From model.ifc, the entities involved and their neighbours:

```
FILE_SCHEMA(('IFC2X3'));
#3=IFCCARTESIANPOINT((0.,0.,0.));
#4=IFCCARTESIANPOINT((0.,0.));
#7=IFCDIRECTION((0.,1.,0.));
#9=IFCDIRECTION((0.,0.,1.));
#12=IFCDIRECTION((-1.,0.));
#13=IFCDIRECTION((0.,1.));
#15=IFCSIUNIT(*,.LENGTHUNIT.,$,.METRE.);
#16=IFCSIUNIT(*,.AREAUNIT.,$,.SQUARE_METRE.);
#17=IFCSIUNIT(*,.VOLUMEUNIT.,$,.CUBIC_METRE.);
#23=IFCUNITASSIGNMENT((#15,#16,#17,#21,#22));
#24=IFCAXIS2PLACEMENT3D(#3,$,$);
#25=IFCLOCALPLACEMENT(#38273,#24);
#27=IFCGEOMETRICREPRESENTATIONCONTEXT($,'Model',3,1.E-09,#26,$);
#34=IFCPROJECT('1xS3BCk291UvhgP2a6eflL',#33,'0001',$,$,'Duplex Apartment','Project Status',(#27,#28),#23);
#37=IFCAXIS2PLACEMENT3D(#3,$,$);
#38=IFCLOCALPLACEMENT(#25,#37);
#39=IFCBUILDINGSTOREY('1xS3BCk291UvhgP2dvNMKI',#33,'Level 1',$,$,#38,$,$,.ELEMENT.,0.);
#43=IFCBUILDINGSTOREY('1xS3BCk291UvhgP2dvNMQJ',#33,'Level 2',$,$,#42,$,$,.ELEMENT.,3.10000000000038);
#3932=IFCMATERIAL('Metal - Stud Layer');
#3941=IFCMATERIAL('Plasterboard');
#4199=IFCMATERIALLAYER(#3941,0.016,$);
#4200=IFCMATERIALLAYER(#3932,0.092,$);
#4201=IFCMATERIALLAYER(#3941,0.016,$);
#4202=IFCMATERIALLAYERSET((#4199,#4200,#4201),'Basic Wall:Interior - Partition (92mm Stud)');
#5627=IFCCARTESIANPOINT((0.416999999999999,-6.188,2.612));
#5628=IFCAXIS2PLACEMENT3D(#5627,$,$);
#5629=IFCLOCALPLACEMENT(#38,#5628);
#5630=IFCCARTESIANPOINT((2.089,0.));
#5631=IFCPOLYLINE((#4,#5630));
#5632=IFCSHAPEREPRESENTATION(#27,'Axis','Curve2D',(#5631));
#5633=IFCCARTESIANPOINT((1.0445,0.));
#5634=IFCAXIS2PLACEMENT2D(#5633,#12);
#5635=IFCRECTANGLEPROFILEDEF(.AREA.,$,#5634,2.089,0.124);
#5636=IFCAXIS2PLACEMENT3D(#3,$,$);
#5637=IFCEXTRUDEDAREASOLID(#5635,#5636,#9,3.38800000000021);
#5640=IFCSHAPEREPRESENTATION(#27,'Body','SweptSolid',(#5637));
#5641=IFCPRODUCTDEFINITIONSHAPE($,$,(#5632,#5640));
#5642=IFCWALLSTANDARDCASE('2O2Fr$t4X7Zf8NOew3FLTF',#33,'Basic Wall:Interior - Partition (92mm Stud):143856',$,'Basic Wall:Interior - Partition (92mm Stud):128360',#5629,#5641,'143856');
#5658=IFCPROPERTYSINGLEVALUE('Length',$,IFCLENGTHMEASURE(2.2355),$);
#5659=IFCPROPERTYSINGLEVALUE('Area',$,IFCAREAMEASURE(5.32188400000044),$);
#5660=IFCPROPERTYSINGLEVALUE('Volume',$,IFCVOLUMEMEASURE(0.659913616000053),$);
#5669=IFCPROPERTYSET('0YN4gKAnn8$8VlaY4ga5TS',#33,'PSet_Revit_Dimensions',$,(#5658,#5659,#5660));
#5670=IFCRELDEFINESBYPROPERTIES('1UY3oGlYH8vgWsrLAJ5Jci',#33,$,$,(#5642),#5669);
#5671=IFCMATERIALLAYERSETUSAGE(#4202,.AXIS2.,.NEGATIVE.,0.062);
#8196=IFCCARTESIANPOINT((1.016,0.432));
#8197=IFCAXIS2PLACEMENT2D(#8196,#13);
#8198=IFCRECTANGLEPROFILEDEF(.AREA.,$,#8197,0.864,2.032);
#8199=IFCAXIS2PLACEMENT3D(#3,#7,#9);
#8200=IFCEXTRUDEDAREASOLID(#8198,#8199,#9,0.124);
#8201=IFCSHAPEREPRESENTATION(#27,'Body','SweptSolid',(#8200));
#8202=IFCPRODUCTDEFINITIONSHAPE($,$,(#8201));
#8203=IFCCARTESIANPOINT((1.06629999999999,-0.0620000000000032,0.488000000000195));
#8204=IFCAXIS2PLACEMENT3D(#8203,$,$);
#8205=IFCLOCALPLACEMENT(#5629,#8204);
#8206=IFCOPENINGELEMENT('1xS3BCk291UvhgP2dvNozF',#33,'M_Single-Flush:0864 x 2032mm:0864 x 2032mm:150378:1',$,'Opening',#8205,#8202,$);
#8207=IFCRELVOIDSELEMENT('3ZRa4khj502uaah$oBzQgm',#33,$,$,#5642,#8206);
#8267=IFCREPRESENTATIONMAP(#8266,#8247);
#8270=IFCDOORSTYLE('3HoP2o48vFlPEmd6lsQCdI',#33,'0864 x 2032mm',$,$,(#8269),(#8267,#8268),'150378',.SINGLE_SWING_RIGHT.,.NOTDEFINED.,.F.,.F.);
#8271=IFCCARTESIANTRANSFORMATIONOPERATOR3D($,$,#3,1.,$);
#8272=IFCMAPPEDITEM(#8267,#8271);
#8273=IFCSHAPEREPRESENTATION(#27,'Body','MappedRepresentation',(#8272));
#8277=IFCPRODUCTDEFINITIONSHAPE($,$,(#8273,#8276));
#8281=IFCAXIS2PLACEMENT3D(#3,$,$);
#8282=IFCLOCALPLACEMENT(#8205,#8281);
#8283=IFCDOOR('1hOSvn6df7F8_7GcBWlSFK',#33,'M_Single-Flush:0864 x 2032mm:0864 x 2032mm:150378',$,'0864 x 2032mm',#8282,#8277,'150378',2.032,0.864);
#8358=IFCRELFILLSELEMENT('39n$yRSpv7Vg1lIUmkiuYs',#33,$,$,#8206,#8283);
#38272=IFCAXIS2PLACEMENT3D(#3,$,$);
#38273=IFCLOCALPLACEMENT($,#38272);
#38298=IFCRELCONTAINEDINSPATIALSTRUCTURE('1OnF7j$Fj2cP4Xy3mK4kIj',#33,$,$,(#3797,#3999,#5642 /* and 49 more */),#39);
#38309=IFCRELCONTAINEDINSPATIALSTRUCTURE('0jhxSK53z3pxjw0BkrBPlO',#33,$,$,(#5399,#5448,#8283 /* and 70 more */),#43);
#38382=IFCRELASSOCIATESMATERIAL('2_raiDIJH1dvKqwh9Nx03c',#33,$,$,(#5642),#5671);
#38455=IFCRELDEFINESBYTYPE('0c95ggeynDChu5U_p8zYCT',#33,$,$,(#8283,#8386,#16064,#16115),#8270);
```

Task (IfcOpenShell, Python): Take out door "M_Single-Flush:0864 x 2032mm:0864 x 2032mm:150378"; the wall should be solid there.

```python
import ifcopenshell
import ifcopenshell.api.feature
import ifcopenshell.api.pset
import ifcopenshell.api.root
import ifcopenshell.geom
import ifcopenshell.util.element
import ifcopenshell.util.shape
import ifcopenshell.util.unit

model = ifcopenshell.open("model.ifc")
area_scale = ifcopenshell.util.unit.calculate_unit_scale(model, "AREAUNIT")
volume_scale = ifcopenshell.util.unit.calculate_unit_scale(model, "VOLUMEUNIT")
settings = ifcopenshell.geom.settings()


def volume(element):
    """Net volume in cubic metres, openings subtracted."""
    shape = ifcopenshell.geom.create_shape(settings, element)
    return ifcopenshell.util.shape.get_volume(shape.geometry)


door = model.by_guid("1hOSvn6df7F8_7GcBWlSFK")
opening = door.FillsVoids[0].RelatingOpeningElement
wall = opening.VoidsElements[0].RelatingBuildingElement
before = volume(wall)

ifcopenshell.api.root.remove_product(model, product=door)
ifcopenshell.api.feature.remove_feature(model, feature=opening)

after = volume(wall)
thickness = 0.124  # wall thickness in metres

# Update the wall's stored quantities.
pset = model.by_id(ifcopenshell.util.element.get_pset(wall, "PSet_Revit_Dimensions", should_inherit=False)["id"])
ifcopenshell.api.pset.edit_pset(model, pset=pset, properties={
    "Area": model.create_entity("IfcAreaMeasure", after / thickness / area_scale),
    "Volume": model.create_entity("IfcVolumeMeasure", after / volume_scale),
})

print(f"wall volume {before:.3f} -> {after:.3f} m3")

model.write("model_updated.ifc")
```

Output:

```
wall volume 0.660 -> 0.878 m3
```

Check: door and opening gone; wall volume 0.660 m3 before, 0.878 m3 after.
